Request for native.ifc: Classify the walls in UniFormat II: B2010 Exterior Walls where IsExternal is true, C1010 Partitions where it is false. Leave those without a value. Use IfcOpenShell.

First a look at what the model holds.

```python
import ifcopenshell
import ifcopenshell.util.element

model = ifcopenshell.open("native.ifc")
print(model.schema)
print("classifications:", [c.Name for c in model.by_type("IfcClassification")])
values = [ifcopenshell.util.element.get_pset(e, "Pset_WallCommon", "IsExternal") for e in model.by_type("IfcWall")]
for value in (True, False, None):
    print("IsExternal", value, values.count(value))
```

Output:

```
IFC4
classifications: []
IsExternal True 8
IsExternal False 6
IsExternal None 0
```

```python
import ifcopenshell
import ifcopenshell.api.classification
import ifcopenshell.util.element

model = ifcopenshell.open("native.ifc")

system = ifcopenshell.api.classification.add_classification(model, classification="UniFormat II")

walls = model.by_type("IfcWall")
external = {e: ifcopenshell.util.element.get_pset(e, "Pset_WallCommon", "IsExternal") for e in walls}
for flag, code, name in ((True, "B2010", "Exterior Walls"), (False, "C1010", "Partitions")):
    products = [e for e in walls if external[e] is flag]
    ifcopenshell.api.classification.add_reference(
        model, products=products, classification=system, identification=code, name=name
    )
    print(code, len(products))

model.write("native_v2.ifc")
```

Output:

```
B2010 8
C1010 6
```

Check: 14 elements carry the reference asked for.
